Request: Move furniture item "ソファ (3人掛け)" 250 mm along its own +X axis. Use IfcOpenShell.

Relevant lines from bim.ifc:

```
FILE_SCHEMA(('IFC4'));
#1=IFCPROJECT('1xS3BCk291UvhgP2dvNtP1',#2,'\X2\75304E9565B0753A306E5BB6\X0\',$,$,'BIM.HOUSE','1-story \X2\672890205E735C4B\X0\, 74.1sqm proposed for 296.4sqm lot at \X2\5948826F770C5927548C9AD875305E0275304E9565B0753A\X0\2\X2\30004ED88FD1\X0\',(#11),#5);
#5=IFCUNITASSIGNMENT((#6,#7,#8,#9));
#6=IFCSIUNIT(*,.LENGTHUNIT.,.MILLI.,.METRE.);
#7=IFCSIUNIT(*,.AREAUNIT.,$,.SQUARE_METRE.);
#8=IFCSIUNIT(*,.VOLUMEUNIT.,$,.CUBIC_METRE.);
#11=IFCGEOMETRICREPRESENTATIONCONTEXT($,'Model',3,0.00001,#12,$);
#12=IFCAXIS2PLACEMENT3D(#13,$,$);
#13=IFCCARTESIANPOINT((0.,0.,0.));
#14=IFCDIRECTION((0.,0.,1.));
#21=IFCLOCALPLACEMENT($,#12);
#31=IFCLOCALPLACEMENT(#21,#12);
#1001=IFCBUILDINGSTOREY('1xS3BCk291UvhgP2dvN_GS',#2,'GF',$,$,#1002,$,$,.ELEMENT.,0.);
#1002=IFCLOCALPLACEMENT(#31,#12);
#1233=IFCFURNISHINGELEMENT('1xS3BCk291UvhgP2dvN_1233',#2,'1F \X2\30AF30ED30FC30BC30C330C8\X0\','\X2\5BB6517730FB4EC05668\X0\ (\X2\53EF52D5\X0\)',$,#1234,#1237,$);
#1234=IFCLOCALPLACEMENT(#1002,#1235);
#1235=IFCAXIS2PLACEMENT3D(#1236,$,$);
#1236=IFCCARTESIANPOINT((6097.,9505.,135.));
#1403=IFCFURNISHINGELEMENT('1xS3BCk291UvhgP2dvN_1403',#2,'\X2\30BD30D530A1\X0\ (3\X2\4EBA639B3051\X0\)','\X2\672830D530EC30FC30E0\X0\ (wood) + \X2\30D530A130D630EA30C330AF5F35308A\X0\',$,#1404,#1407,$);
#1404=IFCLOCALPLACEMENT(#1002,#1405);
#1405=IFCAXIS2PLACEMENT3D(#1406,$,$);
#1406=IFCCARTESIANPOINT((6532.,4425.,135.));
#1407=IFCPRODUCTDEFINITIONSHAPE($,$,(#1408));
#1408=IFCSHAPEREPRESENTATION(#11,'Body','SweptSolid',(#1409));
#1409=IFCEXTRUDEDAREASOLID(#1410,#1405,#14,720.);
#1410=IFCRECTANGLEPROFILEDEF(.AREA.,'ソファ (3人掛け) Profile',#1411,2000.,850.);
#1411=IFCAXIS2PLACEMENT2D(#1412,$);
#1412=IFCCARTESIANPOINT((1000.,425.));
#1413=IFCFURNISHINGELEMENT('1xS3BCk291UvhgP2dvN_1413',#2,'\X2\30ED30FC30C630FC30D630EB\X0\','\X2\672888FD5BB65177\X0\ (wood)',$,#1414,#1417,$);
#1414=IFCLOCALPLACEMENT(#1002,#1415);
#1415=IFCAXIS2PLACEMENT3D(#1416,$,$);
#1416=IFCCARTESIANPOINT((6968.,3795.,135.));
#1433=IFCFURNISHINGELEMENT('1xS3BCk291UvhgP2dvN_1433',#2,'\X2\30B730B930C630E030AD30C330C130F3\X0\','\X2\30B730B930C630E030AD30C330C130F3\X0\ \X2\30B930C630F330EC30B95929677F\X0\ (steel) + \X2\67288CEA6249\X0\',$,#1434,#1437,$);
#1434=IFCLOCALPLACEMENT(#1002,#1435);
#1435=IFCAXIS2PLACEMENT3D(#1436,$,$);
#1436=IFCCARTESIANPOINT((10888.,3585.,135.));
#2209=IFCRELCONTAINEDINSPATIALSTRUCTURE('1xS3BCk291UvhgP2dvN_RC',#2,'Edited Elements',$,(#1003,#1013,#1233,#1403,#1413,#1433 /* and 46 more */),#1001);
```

```python
import ifcopenshell
import ifcopenshell.api.geometry
import ifcopenshell.util.placement
import ifcopenshell.util.unit

model = ifcopenshell.open("bim.ifc")
unit_scale = ifcopenshell.util.unit.calculate_unit_scale(model)

item = model.by_id(1403)
matrix = ifcopenshell.util.placement.get_local_placement(item.ObjectPlacement)
matrix[:3, 3] += matrix[:3, 0] * 0.25 / unit_scale
ifcopenshell.api.geometry.edit_object_placement(model, product=item, matrix=matrix, is_si=False)

print(ifcopenshell.util.placement.get_local_placement(item.ObjectPlacement).round(3) + 0.0)

model.write("bim_updated.ifc")
```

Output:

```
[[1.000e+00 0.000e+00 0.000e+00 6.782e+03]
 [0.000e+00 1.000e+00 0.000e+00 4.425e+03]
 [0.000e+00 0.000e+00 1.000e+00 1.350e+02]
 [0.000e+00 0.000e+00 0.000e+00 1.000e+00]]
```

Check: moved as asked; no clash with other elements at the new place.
